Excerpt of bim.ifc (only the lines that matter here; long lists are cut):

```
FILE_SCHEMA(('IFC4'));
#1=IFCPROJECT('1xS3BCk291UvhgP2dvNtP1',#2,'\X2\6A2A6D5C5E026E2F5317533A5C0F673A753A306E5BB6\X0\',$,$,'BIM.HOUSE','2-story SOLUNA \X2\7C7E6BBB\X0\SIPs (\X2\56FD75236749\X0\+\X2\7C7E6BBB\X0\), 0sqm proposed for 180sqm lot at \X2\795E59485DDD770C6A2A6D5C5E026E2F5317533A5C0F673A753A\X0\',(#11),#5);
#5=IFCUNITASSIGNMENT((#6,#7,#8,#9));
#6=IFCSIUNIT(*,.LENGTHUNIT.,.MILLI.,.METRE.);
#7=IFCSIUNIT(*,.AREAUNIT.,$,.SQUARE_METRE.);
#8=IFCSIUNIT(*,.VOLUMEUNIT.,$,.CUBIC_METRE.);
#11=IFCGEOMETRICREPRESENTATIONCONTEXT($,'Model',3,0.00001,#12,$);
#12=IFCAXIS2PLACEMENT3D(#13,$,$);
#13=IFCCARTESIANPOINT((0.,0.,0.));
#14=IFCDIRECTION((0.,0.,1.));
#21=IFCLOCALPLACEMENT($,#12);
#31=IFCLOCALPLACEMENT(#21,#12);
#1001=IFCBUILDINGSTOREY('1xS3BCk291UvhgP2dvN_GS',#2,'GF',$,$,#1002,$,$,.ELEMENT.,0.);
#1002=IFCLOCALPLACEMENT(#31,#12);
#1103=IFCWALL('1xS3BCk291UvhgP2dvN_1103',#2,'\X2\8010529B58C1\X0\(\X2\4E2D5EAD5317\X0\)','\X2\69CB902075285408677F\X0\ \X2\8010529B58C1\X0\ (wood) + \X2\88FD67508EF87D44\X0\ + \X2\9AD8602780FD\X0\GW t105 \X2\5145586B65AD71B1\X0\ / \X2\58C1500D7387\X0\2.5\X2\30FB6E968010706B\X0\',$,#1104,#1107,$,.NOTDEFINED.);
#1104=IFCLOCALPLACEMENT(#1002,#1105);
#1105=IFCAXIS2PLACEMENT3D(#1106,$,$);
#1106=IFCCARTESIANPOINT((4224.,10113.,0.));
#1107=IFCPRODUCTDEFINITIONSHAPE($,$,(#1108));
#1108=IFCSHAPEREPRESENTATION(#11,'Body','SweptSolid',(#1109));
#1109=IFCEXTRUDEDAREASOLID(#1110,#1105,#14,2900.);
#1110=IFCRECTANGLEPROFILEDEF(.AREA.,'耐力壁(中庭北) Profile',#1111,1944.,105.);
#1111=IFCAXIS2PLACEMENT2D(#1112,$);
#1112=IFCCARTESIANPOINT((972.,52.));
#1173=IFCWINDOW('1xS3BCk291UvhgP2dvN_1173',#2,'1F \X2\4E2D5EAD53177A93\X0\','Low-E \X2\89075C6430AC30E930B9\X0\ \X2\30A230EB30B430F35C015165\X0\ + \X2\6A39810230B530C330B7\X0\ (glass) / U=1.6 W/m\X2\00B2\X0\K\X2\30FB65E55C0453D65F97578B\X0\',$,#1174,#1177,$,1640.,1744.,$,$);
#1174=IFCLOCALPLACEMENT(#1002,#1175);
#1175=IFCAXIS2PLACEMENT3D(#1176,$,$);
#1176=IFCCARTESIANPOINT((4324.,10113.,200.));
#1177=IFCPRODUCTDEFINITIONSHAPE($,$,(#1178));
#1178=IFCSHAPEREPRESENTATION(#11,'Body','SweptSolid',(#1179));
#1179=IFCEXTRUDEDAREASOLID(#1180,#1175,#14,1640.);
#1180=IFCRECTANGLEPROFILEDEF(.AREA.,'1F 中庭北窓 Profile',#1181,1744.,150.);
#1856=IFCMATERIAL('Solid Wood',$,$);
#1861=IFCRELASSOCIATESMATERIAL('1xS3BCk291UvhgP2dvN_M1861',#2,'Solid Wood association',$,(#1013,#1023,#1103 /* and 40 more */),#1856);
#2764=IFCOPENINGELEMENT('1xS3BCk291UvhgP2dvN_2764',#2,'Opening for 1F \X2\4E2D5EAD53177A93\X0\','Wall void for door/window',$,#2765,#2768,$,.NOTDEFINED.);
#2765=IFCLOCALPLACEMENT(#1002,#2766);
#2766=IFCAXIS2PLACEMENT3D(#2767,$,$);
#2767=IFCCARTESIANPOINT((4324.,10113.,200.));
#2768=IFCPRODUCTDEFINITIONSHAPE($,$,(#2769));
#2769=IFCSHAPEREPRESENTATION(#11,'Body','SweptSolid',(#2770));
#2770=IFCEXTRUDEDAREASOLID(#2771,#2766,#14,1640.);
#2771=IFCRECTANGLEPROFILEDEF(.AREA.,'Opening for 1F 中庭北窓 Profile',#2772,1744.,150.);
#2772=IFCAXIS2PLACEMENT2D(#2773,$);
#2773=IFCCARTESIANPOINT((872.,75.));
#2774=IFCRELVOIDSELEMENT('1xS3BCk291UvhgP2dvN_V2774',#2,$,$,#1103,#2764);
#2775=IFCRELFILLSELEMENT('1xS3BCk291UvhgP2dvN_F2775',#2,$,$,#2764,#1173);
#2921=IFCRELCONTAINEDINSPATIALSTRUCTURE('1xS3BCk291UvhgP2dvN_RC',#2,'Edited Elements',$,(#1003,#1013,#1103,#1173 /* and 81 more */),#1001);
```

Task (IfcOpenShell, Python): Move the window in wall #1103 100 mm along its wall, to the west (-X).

```python
import ifcopenshell
import ifcopenshell.api.geometry
import ifcopenshell.util.placement
import ifcopenshell.util.unit

model = ifcopenshell.open("bim.ifc")
unit_scale = ifcopenshell.util.unit.calculate_unit_scale(model)

window = model.by_guid("1xS3BCk291UvhgP2dvN_1173")
opening = window.FillsVoids[0].RelatingOpeningElement
wall = opening.VoidsElements[0].RelatingBuildingElement

wall_matrix = ifcopenshell.util.placement.get_local_placement(wall.ObjectPlacement)
shift = wall_matrix[:3, 0] * -0.1 / unit_scale
before = ifcopenshell.util.placement.get_local_placement(window.ObjectPlacement)[:3, 3].copy()

# The window is not placed relative to its opening, so move both.
for product in (opening, window):
    matrix = ifcopenshell.util.placement.get_local_placement(product.ObjectPlacement)
    matrix[:3, 3] += shift
    ifcopenshell.api.geometry.edit_object_placement(model, product=product, matrix=matrix, is_si=False)

after = ifcopenshell.util.placement.get_local_placement(window.ObjectPlacement)[:3, 3]
print("window moved by", (after - before).round(3) + 0.0)

model.write("bim_rev.ifc")
```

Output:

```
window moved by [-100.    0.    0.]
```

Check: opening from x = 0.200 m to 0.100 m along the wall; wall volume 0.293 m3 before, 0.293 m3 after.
